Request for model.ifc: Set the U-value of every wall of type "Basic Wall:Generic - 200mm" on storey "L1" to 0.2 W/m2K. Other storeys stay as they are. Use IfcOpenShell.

First a look at what the model holds.

```python
import ifcopenshell
import ifcopenshell.util.element

model = ifcopenshell.open("model.ifc")
print(model.schema)
storey = next(s for s in model.by_type("IfcBuildingStorey") if s.Name == "L1")
walls = [e for e in ifcopenshell.util.element.get_decomposition(storey) if e.is_a("IfcWall")]
seen = {}
for e in walls:
    element_type = ifcopenshell.util.element.get_type(e)
    key = (element_type.Name if element_type != e and element_type else None, ifcopenshell.util.element.get_pset(e, "Pset_WallCommon", "ThermalTransmittance"))
    seen[key] = seen.get(key, 0) + 1
for (name, value), count in sorted(seen.items(), key=str):
    print(count, "x", name, "|", value)
```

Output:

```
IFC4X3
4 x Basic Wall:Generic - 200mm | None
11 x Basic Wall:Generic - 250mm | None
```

```python
import ifcopenshell
import ifcopenshell.api.pset
import ifcopenshell.util.element

model = ifcopenshell.open("model.ifc")

storey = next(s for s in model.by_type("IfcBuildingStorey") if s.Name == "L1")
walls = [e for e in ifcopenshell.util.element.get_decomposition(storey) if e.is_a("IfcWall")]

count = 0
for e in walls:
    element_type = ifcopenshell.util.element.get_type(e)
    if element_type in (None, e) or element_type.Name != "Basic Wall:Generic - 200mm":
        continue
    # add_pset returns the element's existing set when there is one.
    pset = ifcopenshell.api.pset.add_pset(model, product=e, name="Pset_WallCommon")
    ifcopenshell.api.pset.edit_pset(model, pset=pset, properties={"ThermalTransmittance": 0.2})
    count += 1

print(count, "walls updated")

model.write("model_rev.ifc")
```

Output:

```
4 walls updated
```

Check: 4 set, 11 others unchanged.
